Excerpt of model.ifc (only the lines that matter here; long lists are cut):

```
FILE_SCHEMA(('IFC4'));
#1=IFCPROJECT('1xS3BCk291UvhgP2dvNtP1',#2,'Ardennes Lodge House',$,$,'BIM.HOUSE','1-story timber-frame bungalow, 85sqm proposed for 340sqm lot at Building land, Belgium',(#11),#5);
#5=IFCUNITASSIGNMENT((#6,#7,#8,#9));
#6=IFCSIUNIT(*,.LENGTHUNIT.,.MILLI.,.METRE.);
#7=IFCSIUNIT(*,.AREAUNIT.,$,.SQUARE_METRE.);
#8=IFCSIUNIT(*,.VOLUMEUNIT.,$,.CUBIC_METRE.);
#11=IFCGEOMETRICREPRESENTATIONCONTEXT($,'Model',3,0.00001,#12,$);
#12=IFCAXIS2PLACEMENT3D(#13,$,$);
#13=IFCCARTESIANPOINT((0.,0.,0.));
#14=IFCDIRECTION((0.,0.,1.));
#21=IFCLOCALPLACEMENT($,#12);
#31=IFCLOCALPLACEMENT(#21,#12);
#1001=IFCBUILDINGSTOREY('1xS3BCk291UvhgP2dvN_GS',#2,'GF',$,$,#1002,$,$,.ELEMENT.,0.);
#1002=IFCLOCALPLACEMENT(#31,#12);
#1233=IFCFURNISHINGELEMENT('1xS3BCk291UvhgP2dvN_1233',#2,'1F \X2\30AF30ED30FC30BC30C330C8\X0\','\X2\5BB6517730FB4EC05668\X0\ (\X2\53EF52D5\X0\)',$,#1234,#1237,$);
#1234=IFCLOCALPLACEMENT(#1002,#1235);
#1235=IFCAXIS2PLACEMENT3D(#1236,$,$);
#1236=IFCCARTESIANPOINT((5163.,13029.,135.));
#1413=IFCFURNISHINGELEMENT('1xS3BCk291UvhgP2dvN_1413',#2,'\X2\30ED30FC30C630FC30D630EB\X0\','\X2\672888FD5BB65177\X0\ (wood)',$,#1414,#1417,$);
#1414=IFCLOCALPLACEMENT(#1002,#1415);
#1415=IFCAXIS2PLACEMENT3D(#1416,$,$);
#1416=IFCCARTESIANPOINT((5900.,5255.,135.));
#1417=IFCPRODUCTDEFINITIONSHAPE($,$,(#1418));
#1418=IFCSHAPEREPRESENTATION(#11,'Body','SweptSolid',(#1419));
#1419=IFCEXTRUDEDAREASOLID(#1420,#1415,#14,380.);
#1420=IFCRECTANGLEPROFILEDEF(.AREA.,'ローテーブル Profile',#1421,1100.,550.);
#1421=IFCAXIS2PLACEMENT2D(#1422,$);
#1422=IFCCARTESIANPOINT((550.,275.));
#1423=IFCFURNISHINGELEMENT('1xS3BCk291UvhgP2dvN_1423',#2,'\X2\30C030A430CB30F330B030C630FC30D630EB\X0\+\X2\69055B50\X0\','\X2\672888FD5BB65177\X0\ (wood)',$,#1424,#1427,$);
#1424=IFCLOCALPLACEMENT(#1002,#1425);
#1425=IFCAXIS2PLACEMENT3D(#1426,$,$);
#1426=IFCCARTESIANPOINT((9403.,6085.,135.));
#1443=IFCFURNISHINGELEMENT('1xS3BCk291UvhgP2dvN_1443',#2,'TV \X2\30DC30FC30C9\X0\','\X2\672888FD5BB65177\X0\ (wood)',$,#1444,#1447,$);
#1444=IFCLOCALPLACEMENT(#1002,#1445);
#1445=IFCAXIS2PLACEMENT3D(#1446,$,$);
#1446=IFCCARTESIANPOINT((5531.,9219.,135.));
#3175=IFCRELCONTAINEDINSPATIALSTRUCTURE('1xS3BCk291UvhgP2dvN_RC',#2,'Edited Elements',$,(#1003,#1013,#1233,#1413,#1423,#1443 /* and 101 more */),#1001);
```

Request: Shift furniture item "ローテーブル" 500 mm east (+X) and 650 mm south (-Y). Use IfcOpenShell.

```python
import ifcopenshell
import ifcopenshell.api.geometry
import ifcopenshell.util.placement
import ifcopenshell.util.unit

model = ifcopenshell.open("model.ifc")
unit_scale = ifcopenshell.util.unit.calculate_unit_scale(model)

item = model.by_id(1413)
matrix = ifcopenshell.util.placement.get_local_placement(item.ObjectPlacement)
matrix[0, 3] += 0.5 / unit_scale
matrix[1, 3] -= 0.65 / unit_scale
ifcopenshell.api.geometry.edit_object_placement(model, product=item, matrix=matrix, is_si=False)

print(ifcopenshell.util.placement.get_local_placement(item.ObjectPlacement).round(3) + 0.0)

model.write("model-out.ifc")
```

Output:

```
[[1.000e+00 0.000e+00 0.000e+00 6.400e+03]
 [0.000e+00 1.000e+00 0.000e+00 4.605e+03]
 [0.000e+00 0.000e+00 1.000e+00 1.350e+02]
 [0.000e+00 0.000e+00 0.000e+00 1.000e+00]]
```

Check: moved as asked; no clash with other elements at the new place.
